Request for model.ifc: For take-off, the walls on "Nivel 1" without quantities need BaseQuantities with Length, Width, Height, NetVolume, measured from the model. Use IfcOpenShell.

First a look at what the model holds.

```python
import ifcopenshell
import ifcopenshell.util.element
import ifcopenshell.util.unit

model = ifcopenshell.open("model.ifc")
print(model.schema)
for unit_type in ("LENGTHUNIT", "AREAUNIT", "VOLUMEUNIT"):
    print(unit_type, ifcopenshell.util.unit.calculate_unit_scale(model, unit_type))
storey = next(s for s in model.by_type("IfcBuildingStorey") if s.Name == "Nivel 1")
walls = [e for e in ifcopenshell.util.element.get_decomposition(storey) if e.is_a("IfcWall")]
for e in sorted(walls, key=lambda e: e.id()):
    print(e.id(), e.is_a(), e.Name, list(ifcopenshell.util.element.get_psets(e, qtos_only=True)), sep=" | ")
```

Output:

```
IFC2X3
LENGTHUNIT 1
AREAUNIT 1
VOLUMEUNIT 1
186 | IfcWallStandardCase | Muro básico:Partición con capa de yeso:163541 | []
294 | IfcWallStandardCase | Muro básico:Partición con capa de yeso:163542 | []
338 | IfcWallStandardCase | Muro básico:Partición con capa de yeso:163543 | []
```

```python
import ifcopenshell
import ifcopenshell.api.pset
import ifcopenshell.geom
import ifcopenshell.util.element
import ifcopenshell.util.shape
import ifcopenshell.util.unit

model = ifcopenshell.open("model.ifc")
unit_scale = ifcopenshell.util.unit.calculate_unit_scale(model)
volume_scale = ifcopenshell.util.unit.calculate_unit_scale(model, "VOLUMEUNIT")
settings = ifcopenshell.geom.settings()

storey = next(s for s in model.by_type("IfcBuildingStorey") if s.Name == "Nivel 1")
walls = [e for e in ifcopenshell.util.element.get_decomposition(storey) if e.is_a("IfcWall")]

for e in sorted(walls, key=lambda e: e.id()):
    if ifcopenshell.util.element.get_psets(e, qtos_only=True, should_inherit=False):
        continue
    # Geometry comes back in metres, in the element's own axes.
    shape = ifcopenshell.geom.create_shape(settings, e)
    values = {
        "Length": ifcopenshell.util.shape.get_x(shape.geometry) / unit_scale,
        "Width": ifcopenshell.util.shape.get_y(shape.geometry) / unit_scale,
        "Height": ifcopenshell.util.shape.get_z(shape.geometry) / unit_scale,
        "NetVolume": ifcopenshell.util.shape.get_volume(shape.geometry) / volume_scale,
    }
    qto = ifcopenshell.api.pset.add_qto(model, product=e, name="BaseQuantities")
    ifcopenshell.api.pset.edit_qto(model, qto=qto, properties=values)
    print(e.id(), {k: round(v, 3) for k, v in values.items()})

model.write("model_rev.ifc")
```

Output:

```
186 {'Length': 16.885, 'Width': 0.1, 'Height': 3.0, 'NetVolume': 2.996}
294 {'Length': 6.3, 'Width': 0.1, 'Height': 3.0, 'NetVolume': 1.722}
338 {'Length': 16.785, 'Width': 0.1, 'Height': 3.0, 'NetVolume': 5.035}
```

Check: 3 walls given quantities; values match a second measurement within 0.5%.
